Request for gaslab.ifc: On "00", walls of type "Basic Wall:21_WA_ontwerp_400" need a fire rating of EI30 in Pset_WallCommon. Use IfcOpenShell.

First a look at what the model holds.

```python
import ifcopenshell
import ifcopenshell.util.element

model = ifcopenshell.open("gaslab.ifc")
print(model.schema)
storey = next(s for s in model.by_type("IfcBuildingStorey") if s.Name == "00")
walls = [e for e in ifcopenshell.util.element.get_decomposition(storey) if e.is_a("IfcWall")]
seen = {}
for e in walls:
    element_type = ifcopenshell.util.element.get_type(e)
    key = (element_type.Name if element_type != e and element_type else None, ifcopenshell.util.element.get_pset(e, "Pset_WallCommon", "FireRating"))
    seen[key] = seen.get(key, 0) + 1
for (name, value), count in sorted(seen.items(), key=str):
    print(count, "x", name, "|", value)
```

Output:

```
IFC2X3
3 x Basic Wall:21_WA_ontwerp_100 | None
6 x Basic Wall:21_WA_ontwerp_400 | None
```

```python
import ifcopenshell
import ifcopenshell.api.pset
import ifcopenshell.util.element

model = ifcopenshell.open("gaslab.ifc")

storey = next(s for s in model.by_type("IfcBuildingStorey") if s.Name == "00")
walls = [e for e in ifcopenshell.util.element.get_decomposition(storey) if e.is_a("IfcWall")]

count = 0
for e in walls:
    element_type = ifcopenshell.util.element.get_type(e)
    if element_type in (None, e) or element_type.Name != "Basic Wall:21_WA_ontwerp_400":
        continue
    # add_pset returns the element's existing set when there is one.
    pset = ifcopenshell.api.pset.add_pset(model, product=e, name="Pset_WallCommon")
    ifcopenshell.api.pset.edit_pset(model, pset=pset, properties={"FireRating": "EI30"})
    count += 1

print(count, "walls updated")

model.write("gaslab_v2.ifc")
```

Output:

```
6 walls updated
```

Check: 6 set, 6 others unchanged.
